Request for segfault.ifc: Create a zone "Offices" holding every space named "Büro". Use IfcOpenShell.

First a look at what the model holds.

```python
import ifcopenshell

model = ifcopenshell.open("segfault.ifc")
print(model.schema)
seen = {}
for space in model.by_type("IfcSpace"):
    seen[space.LongName] = seen.get(space.LongName, 0) + 1
for name, count in sorted(seen.items(), key=str):
    print(count, "x", name)
print("zones:", [z.Name for z in model.by_type("IfcZone")][:20])
```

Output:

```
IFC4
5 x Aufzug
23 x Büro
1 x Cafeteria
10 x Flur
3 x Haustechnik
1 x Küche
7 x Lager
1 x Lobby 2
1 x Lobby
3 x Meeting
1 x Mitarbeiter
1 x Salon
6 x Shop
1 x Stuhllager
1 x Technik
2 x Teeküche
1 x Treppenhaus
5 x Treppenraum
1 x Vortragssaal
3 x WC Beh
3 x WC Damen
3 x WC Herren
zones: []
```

```python
import ifcopenshell
import ifcopenshell.api.group
import ifcopenshell.api.root

model = ifcopenshell.open("segfault.ifc")

names = {"Büro"}
spaces = [s for s in model.by_type("IfcSpace") if s.LongName in names]

zone = ifcopenshell.api.root.create_entity(model, ifc_class="IfcZone", name="Offices")
ifcopenshell.api.group.assign_group(model, products=spaces, group=zone)
print(len(spaces), "spaces in", zone.Name)

model.write("segfault_edited.ifc")
```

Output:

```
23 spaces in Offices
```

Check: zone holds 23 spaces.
